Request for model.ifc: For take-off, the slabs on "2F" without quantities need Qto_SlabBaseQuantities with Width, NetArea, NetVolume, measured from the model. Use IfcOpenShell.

First a look at what the model holds.

```python
import ifcopenshell
import ifcopenshell.util.element
import ifcopenshell.util.unit

model = ifcopenshell.open("model.ifc")
print(model.schema)
for unit_type in ("LENGTHUNIT", "AREAUNIT", "VOLUMEUNIT"):
    print(unit_type, ifcopenshell.util.unit.calculate_unit_scale(model, unit_type))
storey = next(s for s in model.by_type("IfcBuildingStorey") if s.Name == "2F")
slabs = [e for e in ifcopenshell.util.element.get_decomposition(storey) if e.is_a("IfcSlab")]
for e in sorted(slabs, key=lambda e: e.id()):
    print(e.id(), e.is_a(), e.Name, list(ifcopenshell.util.element.get_psets(e, qtos_only=True)), sep=" | ")
```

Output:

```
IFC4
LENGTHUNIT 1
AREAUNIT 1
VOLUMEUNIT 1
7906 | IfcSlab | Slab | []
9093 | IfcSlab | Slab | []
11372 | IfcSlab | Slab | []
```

```python
import ifcopenshell
import ifcopenshell.api.pset
import ifcopenshell.geom
import ifcopenshell.util.element
import ifcopenshell.util.shape
import ifcopenshell.util.unit

model = ifcopenshell.open("model.ifc")
unit_scale = ifcopenshell.util.unit.calculate_unit_scale(model)
area_scale = ifcopenshell.util.unit.calculate_unit_scale(model, "AREAUNIT")
volume_scale = ifcopenshell.util.unit.calculate_unit_scale(model, "VOLUMEUNIT")
settings = ifcopenshell.geom.settings()

storey = next(s for s in model.by_type("IfcBuildingStorey") if s.Name == "2F")
slabs = [e for e in ifcopenshell.util.element.get_decomposition(storey) if e.is_a("IfcSlab")]

for e in sorted(slabs, key=lambda e: e.id()):
    if ifcopenshell.util.element.get_psets(e, qtos_only=True, should_inherit=False):
        continue
    # Geometry comes back in metres, in the element's own axes.
    shape = ifcopenshell.geom.create_shape(settings, e)
    values = {
        "Width": ifcopenshell.util.shape.get_z(shape.geometry) / unit_scale,
        "NetArea": ifcopenshell.util.shape.get_footprint_area(shape.geometry) / area_scale,
        "NetVolume": ifcopenshell.util.shape.get_volume(shape.geometry) / volume_scale,
    }
    qto = ifcopenshell.api.pset.add_qto(model, product=e, name="Qto_SlabBaseQuantities")
    ifcopenshell.api.pset.edit_qto(model, qto=qto, properties=values)
    print(e.id(), {k: round(v, 3) for k, v in values.items()})

model.write("model_v2.ifc")
```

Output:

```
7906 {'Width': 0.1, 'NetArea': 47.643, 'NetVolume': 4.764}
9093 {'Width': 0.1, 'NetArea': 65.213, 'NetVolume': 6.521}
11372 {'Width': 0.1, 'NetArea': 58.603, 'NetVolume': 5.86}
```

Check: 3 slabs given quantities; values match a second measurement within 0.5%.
